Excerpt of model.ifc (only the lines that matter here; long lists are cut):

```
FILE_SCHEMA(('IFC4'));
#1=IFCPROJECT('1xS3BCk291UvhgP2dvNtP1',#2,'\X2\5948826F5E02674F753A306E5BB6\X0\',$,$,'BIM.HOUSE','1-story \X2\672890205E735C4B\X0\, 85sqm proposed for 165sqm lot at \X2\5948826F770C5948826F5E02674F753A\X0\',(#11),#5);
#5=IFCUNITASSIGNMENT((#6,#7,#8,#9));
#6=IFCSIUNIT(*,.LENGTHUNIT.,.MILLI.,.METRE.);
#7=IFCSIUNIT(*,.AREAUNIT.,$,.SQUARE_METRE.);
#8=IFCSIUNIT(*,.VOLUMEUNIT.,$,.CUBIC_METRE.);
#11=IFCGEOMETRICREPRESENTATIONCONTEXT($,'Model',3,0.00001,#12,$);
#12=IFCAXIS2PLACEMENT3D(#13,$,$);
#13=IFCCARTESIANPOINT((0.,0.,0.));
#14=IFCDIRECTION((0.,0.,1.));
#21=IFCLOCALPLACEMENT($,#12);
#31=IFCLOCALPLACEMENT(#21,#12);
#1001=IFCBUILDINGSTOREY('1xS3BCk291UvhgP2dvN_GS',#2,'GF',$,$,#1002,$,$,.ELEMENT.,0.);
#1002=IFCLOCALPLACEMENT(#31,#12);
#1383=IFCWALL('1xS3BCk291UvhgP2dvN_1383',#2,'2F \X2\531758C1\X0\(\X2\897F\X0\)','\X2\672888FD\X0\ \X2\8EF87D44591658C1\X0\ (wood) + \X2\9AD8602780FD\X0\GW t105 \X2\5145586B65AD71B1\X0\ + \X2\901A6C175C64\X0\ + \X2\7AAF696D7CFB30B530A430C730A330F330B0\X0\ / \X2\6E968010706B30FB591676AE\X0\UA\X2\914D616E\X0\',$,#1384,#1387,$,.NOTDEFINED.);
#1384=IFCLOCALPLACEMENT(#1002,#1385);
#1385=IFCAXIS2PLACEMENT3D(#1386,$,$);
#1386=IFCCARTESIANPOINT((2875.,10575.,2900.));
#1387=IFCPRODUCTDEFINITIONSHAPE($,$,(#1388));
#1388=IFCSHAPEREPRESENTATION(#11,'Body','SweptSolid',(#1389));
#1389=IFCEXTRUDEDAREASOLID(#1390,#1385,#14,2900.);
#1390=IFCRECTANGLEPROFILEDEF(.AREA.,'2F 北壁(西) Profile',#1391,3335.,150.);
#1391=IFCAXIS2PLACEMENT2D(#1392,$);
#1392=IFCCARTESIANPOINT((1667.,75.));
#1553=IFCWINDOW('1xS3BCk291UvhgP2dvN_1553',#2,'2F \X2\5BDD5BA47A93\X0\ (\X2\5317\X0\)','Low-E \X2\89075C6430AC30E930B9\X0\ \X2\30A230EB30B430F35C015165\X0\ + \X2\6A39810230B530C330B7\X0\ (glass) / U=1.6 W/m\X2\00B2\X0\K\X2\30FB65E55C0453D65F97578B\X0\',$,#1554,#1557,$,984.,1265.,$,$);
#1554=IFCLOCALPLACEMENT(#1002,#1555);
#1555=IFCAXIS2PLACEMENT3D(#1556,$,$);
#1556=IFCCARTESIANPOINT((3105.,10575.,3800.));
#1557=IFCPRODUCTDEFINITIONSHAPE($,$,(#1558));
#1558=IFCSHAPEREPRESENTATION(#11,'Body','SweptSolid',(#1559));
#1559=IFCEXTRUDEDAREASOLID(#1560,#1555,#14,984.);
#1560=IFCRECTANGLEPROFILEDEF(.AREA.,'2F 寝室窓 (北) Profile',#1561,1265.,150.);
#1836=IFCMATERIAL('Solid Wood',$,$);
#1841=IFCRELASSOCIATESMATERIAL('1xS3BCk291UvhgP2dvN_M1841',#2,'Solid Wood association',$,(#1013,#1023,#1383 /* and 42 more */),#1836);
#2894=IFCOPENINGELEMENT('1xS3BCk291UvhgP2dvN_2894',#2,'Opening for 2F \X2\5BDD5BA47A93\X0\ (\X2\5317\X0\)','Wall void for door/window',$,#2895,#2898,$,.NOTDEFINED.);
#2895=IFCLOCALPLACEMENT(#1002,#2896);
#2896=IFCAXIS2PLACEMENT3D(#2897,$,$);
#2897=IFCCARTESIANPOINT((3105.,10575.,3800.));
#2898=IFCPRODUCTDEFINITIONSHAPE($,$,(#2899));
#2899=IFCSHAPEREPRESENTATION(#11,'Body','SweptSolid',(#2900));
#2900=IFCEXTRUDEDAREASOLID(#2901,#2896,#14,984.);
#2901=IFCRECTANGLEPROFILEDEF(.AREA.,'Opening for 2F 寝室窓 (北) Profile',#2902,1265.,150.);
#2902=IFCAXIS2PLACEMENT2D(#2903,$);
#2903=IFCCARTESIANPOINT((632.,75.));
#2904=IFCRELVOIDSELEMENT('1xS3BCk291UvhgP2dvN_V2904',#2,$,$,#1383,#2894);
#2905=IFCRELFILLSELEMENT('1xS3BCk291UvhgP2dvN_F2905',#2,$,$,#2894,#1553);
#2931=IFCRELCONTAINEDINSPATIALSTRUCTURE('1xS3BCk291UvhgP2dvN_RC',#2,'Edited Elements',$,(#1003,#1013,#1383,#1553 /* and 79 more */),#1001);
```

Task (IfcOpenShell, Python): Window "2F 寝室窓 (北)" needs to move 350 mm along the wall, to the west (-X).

```python
import ifcopenshell
import ifcopenshell.api.geometry
import ifcopenshell.util.placement

model = ifcopenshell.open("model.ifc")

window = model.by_guid("1xS3BCk291UvhgP2dvN_1553")
opening = window.FillsVoids[0].RelatingOpeningElement
wall = opening.VoidsElements[0].RelatingBuildingElement

wall_matrix = ifcopenshell.util.placement.get_local_placement(wall.ObjectPlacement)
shift = wall_matrix[:3, 0] * -350.0
before = ifcopenshell.util.placement.get_local_placement(window.ObjectPlacement)[:3, 3].copy()

# The window is not placed relative to its opening, so move both.
for product in (opening, window):
    matrix = ifcopenshell.util.placement.get_local_placement(product.ObjectPlacement)
    matrix[:3, 3] += shift
    ifcopenshell.api.geometry.edit_object_placement(model, product=product, matrix=matrix, is_si=False)

after = ifcopenshell.util.placement.get_local_placement(window.ObjectPlacement)[:3, 3]
print("window moved by", (after - before).round(3) + 0.0)

model.write("model_rev.ifc")
```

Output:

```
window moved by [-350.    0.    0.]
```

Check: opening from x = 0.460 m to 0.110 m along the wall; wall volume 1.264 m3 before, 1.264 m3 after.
